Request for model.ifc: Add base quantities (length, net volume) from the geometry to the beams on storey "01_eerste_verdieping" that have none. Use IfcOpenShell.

First a look at what the model holds.

```python
import ifcopenshell
import ifcopenshell.util.element
import ifcopenshell.util.unit

model = ifcopenshell.open("model.ifc")
print(model.schema)
for unit_type in ("LENGTHUNIT", "AREAUNIT", "VOLUMEUNIT"):
    print(unit_type, ifcopenshell.util.unit.calculate_unit_scale(model, unit_type))
storey = next(s for s in model.by_type("IfcBuildingStorey") if s.Name == "01_eerste_verdieping")
beams = [e for e in ifcopenshell.util.element.get_decomposition(storey) if e.is_a("IfcBeam")]
for e in sorted(beams, key=lambda e: e.id()):
    print(e.id(), e.is_a(), e.Name, list(ifcopenshell.util.element.get_psets(e, qtos_only=True)), sep=" | ")
```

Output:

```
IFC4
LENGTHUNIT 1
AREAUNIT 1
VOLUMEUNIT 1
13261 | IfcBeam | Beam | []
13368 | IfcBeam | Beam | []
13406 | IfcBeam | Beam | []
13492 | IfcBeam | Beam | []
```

```python
import ifcopenshell
import ifcopenshell.api.pset
import ifcopenshell.geom
import ifcopenshell.util.element
import ifcopenshell.util.shape
import ifcopenshell.util.unit

model = ifcopenshell.open("model.ifc")
unit_scale = ifcopenshell.util.unit.calculate_unit_scale(model)
volume_scale = ifcopenshell.util.unit.calculate_unit_scale(model, "VOLUMEUNIT")
settings = ifcopenshell.geom.settings()

storey = next(s for s in model.by_type("IfcBuildingStorey") if s.Name == "01_eerste_verdieping")
beams = [e for e in ifcopenshell.util.element.get_decomposition(storey) if e.is_a("IfcBeam")]

for e in sorted(beams, key=lambda e: e.id()):
    if ifcopenshell.util.element.get_psets(e, qtos_only=True, should_inherit=False):
        continue
    # Geometry comes back in metres, in the element's own axes.
    shape = ifcopenshell.geom.create_shape(settings, e)
    values = {
        "Length": ifcopenshell.util.shape.get_max_xyz(shape.geometry) / unit_scale,
        "NetVolume": ifcopenshell.util.shape.get_volume(shape.geometry) / volume_scale,
    }
    qto = ifcopenshell.api.pset.add_qto(model, product=e, name="Qto_BeamBaseQuantities")
    ifcopenshell.api.pset.edit_qto(model, qto=qto, properties=values)
    print(e.id(), {k: round(v, 3) for k, v in values.items()})

model.write("model_edited.ifc")
```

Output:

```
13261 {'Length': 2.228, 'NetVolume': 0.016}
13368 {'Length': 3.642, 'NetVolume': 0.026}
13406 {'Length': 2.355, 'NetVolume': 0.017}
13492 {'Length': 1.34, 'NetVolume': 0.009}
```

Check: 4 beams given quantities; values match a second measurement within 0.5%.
